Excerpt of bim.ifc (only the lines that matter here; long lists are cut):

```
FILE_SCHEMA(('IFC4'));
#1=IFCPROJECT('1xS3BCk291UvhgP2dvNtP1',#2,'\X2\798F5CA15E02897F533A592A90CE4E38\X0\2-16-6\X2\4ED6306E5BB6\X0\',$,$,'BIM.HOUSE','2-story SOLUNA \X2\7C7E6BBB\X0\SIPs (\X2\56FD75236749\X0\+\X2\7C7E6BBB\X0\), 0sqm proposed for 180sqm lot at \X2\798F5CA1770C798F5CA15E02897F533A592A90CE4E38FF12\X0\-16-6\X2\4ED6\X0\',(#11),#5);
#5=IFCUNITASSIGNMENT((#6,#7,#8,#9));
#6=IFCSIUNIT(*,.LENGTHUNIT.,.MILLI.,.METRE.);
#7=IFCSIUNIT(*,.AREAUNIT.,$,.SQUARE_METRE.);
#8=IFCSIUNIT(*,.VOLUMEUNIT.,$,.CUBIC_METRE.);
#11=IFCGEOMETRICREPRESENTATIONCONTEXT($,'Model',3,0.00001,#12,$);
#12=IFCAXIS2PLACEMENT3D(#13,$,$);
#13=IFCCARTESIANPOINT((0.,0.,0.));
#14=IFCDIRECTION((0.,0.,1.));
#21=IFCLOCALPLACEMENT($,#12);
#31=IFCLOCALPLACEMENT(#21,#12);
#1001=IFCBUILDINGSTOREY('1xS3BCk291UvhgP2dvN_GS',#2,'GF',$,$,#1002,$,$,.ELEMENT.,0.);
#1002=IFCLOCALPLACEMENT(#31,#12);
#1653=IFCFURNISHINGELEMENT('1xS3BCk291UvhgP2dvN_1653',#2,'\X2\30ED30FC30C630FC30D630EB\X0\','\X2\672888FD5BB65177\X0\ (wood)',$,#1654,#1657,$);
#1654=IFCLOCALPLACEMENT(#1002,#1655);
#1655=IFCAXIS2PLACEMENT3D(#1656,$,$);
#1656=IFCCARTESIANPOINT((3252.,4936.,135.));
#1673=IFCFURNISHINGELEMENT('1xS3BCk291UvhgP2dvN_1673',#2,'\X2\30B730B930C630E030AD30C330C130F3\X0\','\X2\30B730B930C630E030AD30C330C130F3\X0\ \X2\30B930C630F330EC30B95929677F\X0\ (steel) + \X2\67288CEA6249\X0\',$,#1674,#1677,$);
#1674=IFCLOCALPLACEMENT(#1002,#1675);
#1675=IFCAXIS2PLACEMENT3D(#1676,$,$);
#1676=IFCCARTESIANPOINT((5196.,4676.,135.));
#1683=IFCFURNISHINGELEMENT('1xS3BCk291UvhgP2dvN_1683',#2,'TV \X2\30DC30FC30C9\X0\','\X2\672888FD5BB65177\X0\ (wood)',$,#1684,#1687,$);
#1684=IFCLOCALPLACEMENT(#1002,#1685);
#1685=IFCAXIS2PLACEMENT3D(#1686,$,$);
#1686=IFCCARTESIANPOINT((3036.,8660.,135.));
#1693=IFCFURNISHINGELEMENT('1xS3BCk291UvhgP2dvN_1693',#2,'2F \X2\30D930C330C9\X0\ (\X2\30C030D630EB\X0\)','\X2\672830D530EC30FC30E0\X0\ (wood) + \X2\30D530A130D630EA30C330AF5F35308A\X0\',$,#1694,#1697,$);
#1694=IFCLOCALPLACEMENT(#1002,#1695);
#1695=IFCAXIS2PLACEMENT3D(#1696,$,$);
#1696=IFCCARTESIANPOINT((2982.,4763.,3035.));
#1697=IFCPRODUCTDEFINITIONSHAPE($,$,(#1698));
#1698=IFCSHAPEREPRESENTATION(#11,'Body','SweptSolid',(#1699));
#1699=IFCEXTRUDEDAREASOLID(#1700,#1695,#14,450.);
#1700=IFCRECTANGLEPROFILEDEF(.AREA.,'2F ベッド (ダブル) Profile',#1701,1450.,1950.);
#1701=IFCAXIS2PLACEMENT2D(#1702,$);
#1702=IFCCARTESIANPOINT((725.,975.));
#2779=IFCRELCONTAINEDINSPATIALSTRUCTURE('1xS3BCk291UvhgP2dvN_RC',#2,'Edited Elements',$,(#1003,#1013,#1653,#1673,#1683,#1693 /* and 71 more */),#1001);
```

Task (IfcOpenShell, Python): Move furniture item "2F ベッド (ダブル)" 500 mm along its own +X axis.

```python
import ifcopenshell
import ifcopenshell.api.geometry
import ifcopenshell.util.placement

model = ifcopenshell.open("bim.ifc")

item = model.by_id(1693)
matrix = ifcopenshell.util.placement.get_local_placement(item.ObjectPlacement)
matrix[:3, 3] += matrix[:3, 0] * 500.0
ifcopenshell.api.geometry.edit_object_placement(model, product=item, matrix=matrix, is_si=False)

print(ifcopenshell.util.placement.get_local_placement(item.ObjectPlacement).round(3) + 0.0)

model.write("bim_edited.ifc")
```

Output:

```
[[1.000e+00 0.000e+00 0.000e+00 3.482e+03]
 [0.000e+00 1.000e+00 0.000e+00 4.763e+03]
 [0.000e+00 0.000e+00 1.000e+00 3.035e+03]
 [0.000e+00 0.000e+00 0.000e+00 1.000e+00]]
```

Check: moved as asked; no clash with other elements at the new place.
